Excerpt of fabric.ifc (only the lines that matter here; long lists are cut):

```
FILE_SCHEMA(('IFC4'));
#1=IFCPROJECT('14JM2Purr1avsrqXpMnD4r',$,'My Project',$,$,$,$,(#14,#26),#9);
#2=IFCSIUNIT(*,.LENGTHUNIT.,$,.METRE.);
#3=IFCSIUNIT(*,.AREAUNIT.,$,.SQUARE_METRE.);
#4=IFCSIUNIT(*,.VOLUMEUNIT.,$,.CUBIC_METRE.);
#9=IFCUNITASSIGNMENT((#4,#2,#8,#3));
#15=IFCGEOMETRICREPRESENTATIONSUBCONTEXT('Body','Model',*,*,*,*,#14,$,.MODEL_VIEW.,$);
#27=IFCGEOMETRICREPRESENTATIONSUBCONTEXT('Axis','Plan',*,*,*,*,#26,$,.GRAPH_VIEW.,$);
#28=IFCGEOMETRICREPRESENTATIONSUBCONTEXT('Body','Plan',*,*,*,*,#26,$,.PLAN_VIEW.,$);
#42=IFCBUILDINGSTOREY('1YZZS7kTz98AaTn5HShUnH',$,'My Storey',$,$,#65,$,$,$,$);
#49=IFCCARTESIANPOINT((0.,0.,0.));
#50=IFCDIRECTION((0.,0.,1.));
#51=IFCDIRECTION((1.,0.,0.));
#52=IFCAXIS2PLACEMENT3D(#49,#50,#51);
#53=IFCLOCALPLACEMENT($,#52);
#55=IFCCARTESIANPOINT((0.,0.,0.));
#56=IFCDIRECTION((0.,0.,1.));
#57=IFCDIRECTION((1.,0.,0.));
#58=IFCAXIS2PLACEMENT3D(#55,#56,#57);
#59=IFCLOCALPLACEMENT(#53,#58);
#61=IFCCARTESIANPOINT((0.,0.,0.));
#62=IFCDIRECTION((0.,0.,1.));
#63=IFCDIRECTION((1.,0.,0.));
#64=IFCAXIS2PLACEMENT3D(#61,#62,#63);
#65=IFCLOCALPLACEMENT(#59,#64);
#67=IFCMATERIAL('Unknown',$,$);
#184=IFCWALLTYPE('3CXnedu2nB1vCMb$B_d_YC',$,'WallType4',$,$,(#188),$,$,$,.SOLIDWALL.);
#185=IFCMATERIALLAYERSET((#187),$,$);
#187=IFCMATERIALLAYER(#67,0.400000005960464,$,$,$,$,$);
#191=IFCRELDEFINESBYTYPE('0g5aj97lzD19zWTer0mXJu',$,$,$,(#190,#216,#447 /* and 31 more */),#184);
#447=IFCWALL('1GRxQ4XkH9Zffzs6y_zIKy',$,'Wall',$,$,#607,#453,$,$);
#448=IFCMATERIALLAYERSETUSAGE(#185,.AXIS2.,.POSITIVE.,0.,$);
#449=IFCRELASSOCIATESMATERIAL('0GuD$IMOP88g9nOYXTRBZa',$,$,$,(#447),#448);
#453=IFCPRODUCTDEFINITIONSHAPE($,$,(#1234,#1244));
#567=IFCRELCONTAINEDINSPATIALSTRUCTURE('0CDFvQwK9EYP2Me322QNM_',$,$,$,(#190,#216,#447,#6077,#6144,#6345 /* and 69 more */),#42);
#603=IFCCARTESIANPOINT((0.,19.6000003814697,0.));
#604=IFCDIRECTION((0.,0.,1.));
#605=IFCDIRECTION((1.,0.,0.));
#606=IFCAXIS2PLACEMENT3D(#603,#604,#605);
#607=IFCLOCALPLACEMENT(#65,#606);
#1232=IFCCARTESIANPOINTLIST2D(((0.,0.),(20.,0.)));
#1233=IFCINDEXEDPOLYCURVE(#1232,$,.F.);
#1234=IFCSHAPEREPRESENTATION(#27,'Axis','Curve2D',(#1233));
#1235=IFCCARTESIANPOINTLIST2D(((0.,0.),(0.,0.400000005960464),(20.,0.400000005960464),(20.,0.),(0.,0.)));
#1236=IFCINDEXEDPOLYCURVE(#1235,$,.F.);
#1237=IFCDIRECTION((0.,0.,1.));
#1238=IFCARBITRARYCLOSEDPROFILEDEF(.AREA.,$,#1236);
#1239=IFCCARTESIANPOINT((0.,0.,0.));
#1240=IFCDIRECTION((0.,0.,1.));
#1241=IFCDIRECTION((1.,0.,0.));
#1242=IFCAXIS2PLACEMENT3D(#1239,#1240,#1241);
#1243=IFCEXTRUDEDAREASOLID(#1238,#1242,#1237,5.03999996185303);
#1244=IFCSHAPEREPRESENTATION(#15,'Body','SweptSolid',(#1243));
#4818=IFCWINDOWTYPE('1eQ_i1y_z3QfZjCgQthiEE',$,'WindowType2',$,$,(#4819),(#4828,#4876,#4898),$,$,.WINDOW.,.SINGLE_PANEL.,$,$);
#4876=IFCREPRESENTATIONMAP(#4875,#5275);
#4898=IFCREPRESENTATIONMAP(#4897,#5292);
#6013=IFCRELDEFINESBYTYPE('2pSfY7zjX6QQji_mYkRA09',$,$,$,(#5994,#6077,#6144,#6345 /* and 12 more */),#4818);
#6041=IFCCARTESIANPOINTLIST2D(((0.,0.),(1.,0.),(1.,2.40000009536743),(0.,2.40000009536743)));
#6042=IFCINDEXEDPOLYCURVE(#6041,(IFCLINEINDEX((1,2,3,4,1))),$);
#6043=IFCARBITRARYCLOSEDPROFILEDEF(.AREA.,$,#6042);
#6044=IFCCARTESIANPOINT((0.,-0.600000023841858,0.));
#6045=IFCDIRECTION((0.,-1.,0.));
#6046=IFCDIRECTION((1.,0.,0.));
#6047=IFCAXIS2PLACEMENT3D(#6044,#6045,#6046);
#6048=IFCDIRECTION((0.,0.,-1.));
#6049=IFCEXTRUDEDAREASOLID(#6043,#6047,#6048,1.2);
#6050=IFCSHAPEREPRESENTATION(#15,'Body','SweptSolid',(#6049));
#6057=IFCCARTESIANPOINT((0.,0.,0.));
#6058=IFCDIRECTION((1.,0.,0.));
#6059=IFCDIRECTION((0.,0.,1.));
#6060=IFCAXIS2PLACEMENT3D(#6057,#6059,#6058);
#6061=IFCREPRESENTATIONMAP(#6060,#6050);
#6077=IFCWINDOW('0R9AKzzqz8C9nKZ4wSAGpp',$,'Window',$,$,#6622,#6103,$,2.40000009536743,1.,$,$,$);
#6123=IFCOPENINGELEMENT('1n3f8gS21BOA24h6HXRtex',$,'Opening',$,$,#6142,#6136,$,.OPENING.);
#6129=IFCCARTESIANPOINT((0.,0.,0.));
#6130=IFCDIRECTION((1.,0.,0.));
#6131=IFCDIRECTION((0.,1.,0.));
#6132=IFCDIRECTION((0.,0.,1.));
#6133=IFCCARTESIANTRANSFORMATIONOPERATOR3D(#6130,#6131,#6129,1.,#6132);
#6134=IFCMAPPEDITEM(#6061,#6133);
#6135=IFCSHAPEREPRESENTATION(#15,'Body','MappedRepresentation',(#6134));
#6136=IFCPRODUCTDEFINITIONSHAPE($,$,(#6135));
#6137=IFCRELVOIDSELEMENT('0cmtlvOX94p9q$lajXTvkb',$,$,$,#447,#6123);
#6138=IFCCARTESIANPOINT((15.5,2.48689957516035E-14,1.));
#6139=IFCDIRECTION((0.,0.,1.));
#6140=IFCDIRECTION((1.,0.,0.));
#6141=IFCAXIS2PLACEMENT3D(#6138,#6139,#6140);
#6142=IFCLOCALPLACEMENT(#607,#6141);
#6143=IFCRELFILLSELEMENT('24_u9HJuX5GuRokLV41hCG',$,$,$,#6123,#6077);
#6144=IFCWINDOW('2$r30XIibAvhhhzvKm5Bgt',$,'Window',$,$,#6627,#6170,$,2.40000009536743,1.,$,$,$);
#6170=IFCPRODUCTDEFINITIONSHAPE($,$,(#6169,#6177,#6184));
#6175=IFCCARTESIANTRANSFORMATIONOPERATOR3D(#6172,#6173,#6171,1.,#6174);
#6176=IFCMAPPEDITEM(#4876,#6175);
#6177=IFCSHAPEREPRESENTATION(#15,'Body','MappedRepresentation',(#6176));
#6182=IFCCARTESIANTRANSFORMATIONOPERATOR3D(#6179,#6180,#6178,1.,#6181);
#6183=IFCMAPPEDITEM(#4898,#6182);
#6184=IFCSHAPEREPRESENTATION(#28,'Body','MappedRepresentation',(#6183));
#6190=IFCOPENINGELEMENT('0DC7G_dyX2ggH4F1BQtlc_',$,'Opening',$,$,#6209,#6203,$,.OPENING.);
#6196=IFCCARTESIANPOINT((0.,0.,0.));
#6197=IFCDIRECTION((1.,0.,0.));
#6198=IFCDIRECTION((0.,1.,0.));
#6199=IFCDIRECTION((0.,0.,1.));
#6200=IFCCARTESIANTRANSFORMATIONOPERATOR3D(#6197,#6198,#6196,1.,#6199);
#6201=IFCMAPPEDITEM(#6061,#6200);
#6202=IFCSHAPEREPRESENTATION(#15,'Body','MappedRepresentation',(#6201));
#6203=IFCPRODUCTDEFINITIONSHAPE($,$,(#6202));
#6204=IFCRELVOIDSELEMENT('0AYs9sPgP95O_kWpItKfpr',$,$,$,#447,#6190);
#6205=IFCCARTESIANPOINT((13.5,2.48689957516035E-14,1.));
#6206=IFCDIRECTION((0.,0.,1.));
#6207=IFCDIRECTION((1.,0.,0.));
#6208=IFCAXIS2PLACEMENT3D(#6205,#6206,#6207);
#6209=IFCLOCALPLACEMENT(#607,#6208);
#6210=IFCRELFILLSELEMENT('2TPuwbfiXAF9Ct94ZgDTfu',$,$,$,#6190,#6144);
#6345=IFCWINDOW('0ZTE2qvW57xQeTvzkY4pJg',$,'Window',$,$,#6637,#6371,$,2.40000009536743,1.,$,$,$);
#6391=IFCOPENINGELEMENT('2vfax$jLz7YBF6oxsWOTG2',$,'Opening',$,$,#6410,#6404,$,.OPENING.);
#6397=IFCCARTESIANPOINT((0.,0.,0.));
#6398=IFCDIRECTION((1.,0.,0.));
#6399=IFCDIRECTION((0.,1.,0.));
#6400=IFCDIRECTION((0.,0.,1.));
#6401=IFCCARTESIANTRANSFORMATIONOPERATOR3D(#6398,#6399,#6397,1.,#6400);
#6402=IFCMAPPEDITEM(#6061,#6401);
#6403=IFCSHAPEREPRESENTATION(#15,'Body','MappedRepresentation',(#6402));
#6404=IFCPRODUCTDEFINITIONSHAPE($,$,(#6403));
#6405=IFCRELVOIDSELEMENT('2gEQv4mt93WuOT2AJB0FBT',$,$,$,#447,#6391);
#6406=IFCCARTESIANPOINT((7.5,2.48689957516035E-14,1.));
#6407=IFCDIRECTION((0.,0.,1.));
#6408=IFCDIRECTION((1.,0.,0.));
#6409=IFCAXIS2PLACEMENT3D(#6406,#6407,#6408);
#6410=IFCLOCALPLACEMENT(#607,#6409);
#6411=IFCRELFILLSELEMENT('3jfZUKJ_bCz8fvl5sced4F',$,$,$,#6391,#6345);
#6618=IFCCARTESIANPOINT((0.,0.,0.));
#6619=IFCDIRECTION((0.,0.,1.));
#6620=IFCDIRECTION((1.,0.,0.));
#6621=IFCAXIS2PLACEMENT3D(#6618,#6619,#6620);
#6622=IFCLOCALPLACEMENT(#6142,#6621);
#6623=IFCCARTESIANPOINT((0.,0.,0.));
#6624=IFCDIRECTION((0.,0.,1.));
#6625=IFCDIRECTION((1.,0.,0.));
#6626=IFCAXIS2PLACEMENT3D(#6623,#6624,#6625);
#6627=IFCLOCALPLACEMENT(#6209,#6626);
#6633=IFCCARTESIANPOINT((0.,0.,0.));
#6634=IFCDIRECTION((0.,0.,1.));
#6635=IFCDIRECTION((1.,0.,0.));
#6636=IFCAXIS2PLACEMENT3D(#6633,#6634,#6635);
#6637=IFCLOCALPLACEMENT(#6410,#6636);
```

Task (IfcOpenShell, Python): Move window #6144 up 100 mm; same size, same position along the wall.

```python
import numpy as np
import ifcopenshell
import ifcopenshell.api.geometry
import ifcopenshell.util.placement
import ifcopenshell.util.unit

model = ifcopenshell.open("fabric.ifc")
unit_scale = ifcopenshell.util.unit.calculate_unit_scale(model)

window = model.by_guid("2$r30XIibAvhhhzvKm5Bgt")
opening = window.FillsVoids[0].RelatingOpeningElement
dz = 0.1 / unit_scale

shift = np.array([0.0, 0.0, dz])
# The window is placed relative to its opening, so it follows when the opening moves.
matrix = ifcopenshell.util.placement.get_local_placement(opening.ObjectPlacement)
matrix[:3, 3] += shift
ifcopenshell.api.geometry.edit_object_placement(
    model, product=opening, matrix=matrix, is_si=False, should_transform_children=True
)

print(f"moved by {dz * unit_scale:+.3f} m")

model.write("fabric_v2.ifc")
```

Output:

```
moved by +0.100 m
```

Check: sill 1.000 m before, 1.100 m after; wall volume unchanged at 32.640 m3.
